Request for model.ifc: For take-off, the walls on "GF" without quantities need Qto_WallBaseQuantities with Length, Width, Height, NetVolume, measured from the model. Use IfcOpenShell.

First a look at what the model holds.

```python
import ifcopenshell
import ifcopenshell.util.element
import ifcopenshell.util.unit

model = ifcopenshell.open("model.ifc")
print(model.schema)
for unit_type in ("LENGTHUNIT", "AREAUNIT", "VOLUMEUNIT"):
    print(unit_type, ifcopenshell.util.unit.calculate_unit_scale(model, unit_type))
storey = next(s for s in model.by_type("IfcBuildingStorey") if s.Name == "GF")
walls = [e for e in ifcopenshell.util.element.get_decomposition(storey) if e.is_a("IfcWall")]
for e in sorted(walls, key=lambda e: e.id()):
    print(e.id(), e.is_a(), e.Name, list(ifcopenshell.util.element.get_psets(e, qtos_only=True)), sep=" | ")
```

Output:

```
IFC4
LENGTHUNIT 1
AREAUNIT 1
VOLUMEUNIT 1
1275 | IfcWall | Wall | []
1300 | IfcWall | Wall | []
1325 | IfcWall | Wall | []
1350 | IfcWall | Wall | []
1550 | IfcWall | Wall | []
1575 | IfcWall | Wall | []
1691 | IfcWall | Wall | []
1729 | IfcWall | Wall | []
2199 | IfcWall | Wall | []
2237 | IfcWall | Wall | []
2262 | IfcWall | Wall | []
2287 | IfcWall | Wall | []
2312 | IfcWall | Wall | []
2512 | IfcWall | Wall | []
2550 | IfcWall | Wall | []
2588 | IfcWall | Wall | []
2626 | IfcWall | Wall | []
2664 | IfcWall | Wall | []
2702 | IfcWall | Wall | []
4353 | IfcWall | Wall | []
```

```python
import ifcopenshell
import ifcopenshell.api.pset
import ifcopenshell.geom
import ifcopenshell.util.element
import ifcopenshell.util.shape
import ifcopenshell.util.unit

model = ifcopenshell.open("model.ifc")
unit_scale = ifcopenshell.util.unit.calculate_unit_scale(model)
volume_scale = ifcopenshell.util.unit.calculate_unit_scale(model, "VOLUMEUNIT")
settings = ifcopenshell.geom.settings()

storey = next(s for s in model.by_type("IfcBuildingStorey") if s.Name == "GF")
walls = [e for e in ifcopenshell.util.element.get_decomposition(storey) if e.is_a("IfcWall")]

for e in sorted(walls, key=lambda e: e.id()):
    if ifcopenshell.util.element.get_psets(e, qtos_only=True, should_inherit=False):
        continue
    # Geometry comes back in metres, in the element's own axes.
    shape = ifcopenshell.geom.create_shape(settings, e)
    values = {
        "Length": ifcopenshell.util.shape.get_x(shape.geometry) / unit_scale,
        "Width": ifcopenshell.util.shape.get_y(shape.geometry) / unit_scale,
        "Height": ifcopenshell.util.shape.get_z(shape.geometry) / unit_scale,
        "NetVolume": ifcopenshell.util.shape.get_volume(shape.geometry) / volume_scale,
    }
    qto = ifcopenshell.api.pset.add_qto(model, product=e, name="Qto_WallBaseQuantities")
    ifcopenshell.api.pset.edit_qto(model, qto=qto, properties=values)
    print(e.id(), {k: round(v, 3) for k, v in values.items()})

model.write("model-out.ifc")
```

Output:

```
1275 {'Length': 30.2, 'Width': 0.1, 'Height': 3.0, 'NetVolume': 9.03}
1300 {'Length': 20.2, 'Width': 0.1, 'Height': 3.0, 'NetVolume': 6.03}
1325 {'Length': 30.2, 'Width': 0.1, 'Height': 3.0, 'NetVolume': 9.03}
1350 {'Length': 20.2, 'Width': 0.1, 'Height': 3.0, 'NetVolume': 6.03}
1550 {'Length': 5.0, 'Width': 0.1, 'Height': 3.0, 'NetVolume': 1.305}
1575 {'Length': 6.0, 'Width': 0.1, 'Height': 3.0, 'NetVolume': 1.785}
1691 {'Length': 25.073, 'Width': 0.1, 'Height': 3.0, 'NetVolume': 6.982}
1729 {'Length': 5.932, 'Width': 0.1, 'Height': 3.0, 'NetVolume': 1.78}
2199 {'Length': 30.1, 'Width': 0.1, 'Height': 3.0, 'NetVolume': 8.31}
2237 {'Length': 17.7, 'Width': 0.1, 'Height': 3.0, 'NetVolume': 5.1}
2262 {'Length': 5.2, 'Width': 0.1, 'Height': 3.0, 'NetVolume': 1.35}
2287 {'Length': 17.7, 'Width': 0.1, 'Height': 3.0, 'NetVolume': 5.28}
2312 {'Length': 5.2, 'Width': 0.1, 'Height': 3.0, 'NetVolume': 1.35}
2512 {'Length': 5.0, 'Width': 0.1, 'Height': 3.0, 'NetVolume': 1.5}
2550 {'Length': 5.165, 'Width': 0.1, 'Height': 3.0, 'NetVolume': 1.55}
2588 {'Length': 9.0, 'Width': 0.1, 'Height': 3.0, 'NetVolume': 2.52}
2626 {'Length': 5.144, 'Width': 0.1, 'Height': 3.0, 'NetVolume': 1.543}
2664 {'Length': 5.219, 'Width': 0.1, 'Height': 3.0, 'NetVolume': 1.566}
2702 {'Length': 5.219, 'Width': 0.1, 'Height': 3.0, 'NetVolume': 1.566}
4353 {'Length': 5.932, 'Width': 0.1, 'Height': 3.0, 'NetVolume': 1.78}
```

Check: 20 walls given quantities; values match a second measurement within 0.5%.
